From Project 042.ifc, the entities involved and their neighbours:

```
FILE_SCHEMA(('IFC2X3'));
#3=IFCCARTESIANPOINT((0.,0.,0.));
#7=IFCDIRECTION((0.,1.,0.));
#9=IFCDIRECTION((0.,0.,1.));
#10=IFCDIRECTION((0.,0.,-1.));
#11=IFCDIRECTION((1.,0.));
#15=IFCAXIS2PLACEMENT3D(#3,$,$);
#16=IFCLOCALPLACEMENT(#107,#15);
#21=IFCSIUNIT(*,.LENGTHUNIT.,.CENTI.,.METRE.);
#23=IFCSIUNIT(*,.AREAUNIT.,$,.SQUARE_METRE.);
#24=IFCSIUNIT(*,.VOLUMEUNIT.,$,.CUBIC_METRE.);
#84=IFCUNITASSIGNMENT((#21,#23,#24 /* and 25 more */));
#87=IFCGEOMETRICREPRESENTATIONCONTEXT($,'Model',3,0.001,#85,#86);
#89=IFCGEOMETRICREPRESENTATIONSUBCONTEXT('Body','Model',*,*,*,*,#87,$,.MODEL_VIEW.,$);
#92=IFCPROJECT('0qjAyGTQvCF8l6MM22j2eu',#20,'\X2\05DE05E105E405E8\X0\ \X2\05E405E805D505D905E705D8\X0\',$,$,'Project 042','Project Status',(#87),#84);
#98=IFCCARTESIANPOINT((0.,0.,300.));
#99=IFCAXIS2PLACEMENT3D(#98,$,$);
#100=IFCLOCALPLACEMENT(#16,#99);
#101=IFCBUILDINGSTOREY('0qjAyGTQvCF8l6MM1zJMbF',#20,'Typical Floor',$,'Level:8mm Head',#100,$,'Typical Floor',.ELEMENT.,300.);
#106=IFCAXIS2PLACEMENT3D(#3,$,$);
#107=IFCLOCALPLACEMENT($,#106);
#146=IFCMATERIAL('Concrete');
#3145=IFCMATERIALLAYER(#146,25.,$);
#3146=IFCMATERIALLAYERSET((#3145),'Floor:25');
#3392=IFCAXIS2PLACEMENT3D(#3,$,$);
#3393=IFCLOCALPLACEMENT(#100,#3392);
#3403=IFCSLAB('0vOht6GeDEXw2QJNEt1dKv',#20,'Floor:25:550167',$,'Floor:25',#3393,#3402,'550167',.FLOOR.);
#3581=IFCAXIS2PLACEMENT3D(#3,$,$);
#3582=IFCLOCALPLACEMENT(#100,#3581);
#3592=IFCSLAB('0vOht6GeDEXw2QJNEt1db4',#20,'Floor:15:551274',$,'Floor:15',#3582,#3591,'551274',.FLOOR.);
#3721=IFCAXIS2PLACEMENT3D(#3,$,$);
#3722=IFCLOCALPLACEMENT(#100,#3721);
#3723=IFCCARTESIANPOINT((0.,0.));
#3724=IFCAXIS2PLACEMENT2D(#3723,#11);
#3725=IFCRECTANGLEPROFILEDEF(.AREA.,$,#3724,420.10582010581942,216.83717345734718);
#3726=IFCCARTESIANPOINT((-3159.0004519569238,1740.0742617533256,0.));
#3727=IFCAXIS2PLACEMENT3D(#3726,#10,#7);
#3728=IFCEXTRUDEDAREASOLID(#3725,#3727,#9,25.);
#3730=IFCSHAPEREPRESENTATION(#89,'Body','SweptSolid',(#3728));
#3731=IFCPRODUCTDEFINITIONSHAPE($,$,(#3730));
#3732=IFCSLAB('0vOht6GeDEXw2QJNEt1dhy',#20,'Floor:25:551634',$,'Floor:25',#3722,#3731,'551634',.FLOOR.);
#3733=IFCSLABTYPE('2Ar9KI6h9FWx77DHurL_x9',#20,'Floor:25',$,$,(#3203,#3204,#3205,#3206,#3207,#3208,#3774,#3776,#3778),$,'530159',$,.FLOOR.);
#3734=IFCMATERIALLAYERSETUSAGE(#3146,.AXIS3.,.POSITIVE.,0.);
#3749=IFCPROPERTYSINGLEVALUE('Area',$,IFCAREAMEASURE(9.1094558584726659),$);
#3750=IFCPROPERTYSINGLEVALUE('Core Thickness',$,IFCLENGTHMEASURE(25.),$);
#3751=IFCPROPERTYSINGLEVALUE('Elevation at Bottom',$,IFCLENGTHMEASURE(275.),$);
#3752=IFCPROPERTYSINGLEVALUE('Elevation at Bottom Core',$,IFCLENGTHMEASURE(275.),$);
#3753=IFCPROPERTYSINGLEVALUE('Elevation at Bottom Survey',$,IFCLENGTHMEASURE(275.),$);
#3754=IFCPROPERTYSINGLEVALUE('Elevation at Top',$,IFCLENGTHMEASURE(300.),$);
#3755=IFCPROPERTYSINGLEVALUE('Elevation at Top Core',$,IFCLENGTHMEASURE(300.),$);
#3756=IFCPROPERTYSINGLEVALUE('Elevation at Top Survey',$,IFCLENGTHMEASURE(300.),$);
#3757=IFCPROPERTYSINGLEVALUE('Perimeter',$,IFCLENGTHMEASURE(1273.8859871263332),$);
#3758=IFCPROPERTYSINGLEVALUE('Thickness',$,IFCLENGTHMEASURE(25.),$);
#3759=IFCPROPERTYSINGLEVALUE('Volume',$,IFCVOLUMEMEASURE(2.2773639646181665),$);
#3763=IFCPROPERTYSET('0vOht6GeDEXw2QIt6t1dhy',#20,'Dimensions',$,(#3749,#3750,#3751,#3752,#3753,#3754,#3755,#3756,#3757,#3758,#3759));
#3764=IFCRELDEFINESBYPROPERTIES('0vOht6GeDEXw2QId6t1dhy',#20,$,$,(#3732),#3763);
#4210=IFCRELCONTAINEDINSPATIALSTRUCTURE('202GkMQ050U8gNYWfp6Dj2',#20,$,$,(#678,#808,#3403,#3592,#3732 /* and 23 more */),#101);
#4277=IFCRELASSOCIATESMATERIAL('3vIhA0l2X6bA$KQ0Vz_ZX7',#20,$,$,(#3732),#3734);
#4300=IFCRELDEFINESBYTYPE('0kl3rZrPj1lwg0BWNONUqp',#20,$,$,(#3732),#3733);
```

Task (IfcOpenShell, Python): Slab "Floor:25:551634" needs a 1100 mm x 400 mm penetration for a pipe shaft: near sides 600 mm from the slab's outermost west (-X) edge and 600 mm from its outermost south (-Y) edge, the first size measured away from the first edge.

```python
import numpy as np
import ifcopenshell
import ifcopenshell.api.feature
import ifcopenshell.api.geometry
import ifcopenshell.api.pset
import ifcopenshell.api.root
import ifcopenshell.geom
import ifcopenshell.util.element
import ifcopenshell.util.placement
import ifcopenshell.util.representation
import ifcopenshell.util.shape
import ifcopenshell.util.unit

model = ifcopenshell.open("Project 042.ifc")
unit_scale = ifcopenshell.util.unit.calculate_unit_scale(model)
area_scale = ifcopenshell.util.unit.calculate_unit_scale(model, "AREAUNIT")
volume_scale = ifcopenshell.util.unit.calculate_unit_scale(model, "VOLUMEUNIT")
settings = ifcopenshell.geom.settings()


def volume(element):
    """Net volume in cubic metres, openings subtracted."""
    shape = ifcopenshell.geom.create_shape(settings, element)
    return ifcopenshell.util.shape.get_volume(shape.geometry)


slab = model.by_guid("0vOht6GeDEXw2QJNEt1dhy")
before = volume(slab)

# Extent in the slab's own axes, in metres. The edges named are its -X and -Y sides.
slab_shape = ifcopenshell.geom.create_shape(settings, slab)
vertices = ifcopenshell.util.shape.get_vertices(slab_shape.geometry)
x_min, y_min, bottom = vertices.min(axis=0)
top = vertices[:, 2].max()

opening = ifcopenshell.api.root.create_entity(model, ifc_class="IfcOpeningElement", name="Pipe shaft opening")
context = ifcopenshell.util.representation.get_context(model, "Model", "Body", "MODEL_VIEW")
width, depth = 1.1, 0.4
outline = [(0.0, 0.0), (width, 0.0), (width, depth), (0.0, depth), (0.0, 0.0)]
# Overshoot both faces by 50 mm so the cut is clean.
shape = ifcopenshell.api.geometry.add_slab_representation(
    model, context=context, depth=top - bottom + 0.1, polyline=outline
)
ifcopenshell.api.geometry.assign_representation(model, product=opening, representation=shape)

matrix = ifcopenshell.util.placement.get_local_placement(slab.ObjectPlacement)
matrix[:, 3] = matrix @ np.append(np.array([x_min + 0.6, y_min + 0.6, bottom - 0.05]) / unit_scale, 1.0)
ifcopenshell.api.geometry.edit_object_placement(model, product=opening, matrix=matrix, is_si=False)
ifcopenshell.api.feature.add_feature(model, feature=opening, element=slab)

after = volume(slab)

# Update the slab's stored quantities.
pset = model.by_id(ifcopenshell.util.element.get_pset(slab, "Dimensions", should_inherit=False)["id"])
ifcopenshell.api.pset.edit_pset(model, pset=pset, properties={
    "Area": model.create_entity("IfcAreaMeasure", after / (top - bottom) / area_scale),
    "Volume": model.create_entity("IfcVolumeMeasure", after / volume_scale),
})

print(f"slab volume {before:.3f} -> {after:.3f} m3")

model.write("Project 042_updated.ifc")
```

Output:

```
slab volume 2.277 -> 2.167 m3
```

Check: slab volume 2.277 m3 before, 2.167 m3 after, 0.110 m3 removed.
